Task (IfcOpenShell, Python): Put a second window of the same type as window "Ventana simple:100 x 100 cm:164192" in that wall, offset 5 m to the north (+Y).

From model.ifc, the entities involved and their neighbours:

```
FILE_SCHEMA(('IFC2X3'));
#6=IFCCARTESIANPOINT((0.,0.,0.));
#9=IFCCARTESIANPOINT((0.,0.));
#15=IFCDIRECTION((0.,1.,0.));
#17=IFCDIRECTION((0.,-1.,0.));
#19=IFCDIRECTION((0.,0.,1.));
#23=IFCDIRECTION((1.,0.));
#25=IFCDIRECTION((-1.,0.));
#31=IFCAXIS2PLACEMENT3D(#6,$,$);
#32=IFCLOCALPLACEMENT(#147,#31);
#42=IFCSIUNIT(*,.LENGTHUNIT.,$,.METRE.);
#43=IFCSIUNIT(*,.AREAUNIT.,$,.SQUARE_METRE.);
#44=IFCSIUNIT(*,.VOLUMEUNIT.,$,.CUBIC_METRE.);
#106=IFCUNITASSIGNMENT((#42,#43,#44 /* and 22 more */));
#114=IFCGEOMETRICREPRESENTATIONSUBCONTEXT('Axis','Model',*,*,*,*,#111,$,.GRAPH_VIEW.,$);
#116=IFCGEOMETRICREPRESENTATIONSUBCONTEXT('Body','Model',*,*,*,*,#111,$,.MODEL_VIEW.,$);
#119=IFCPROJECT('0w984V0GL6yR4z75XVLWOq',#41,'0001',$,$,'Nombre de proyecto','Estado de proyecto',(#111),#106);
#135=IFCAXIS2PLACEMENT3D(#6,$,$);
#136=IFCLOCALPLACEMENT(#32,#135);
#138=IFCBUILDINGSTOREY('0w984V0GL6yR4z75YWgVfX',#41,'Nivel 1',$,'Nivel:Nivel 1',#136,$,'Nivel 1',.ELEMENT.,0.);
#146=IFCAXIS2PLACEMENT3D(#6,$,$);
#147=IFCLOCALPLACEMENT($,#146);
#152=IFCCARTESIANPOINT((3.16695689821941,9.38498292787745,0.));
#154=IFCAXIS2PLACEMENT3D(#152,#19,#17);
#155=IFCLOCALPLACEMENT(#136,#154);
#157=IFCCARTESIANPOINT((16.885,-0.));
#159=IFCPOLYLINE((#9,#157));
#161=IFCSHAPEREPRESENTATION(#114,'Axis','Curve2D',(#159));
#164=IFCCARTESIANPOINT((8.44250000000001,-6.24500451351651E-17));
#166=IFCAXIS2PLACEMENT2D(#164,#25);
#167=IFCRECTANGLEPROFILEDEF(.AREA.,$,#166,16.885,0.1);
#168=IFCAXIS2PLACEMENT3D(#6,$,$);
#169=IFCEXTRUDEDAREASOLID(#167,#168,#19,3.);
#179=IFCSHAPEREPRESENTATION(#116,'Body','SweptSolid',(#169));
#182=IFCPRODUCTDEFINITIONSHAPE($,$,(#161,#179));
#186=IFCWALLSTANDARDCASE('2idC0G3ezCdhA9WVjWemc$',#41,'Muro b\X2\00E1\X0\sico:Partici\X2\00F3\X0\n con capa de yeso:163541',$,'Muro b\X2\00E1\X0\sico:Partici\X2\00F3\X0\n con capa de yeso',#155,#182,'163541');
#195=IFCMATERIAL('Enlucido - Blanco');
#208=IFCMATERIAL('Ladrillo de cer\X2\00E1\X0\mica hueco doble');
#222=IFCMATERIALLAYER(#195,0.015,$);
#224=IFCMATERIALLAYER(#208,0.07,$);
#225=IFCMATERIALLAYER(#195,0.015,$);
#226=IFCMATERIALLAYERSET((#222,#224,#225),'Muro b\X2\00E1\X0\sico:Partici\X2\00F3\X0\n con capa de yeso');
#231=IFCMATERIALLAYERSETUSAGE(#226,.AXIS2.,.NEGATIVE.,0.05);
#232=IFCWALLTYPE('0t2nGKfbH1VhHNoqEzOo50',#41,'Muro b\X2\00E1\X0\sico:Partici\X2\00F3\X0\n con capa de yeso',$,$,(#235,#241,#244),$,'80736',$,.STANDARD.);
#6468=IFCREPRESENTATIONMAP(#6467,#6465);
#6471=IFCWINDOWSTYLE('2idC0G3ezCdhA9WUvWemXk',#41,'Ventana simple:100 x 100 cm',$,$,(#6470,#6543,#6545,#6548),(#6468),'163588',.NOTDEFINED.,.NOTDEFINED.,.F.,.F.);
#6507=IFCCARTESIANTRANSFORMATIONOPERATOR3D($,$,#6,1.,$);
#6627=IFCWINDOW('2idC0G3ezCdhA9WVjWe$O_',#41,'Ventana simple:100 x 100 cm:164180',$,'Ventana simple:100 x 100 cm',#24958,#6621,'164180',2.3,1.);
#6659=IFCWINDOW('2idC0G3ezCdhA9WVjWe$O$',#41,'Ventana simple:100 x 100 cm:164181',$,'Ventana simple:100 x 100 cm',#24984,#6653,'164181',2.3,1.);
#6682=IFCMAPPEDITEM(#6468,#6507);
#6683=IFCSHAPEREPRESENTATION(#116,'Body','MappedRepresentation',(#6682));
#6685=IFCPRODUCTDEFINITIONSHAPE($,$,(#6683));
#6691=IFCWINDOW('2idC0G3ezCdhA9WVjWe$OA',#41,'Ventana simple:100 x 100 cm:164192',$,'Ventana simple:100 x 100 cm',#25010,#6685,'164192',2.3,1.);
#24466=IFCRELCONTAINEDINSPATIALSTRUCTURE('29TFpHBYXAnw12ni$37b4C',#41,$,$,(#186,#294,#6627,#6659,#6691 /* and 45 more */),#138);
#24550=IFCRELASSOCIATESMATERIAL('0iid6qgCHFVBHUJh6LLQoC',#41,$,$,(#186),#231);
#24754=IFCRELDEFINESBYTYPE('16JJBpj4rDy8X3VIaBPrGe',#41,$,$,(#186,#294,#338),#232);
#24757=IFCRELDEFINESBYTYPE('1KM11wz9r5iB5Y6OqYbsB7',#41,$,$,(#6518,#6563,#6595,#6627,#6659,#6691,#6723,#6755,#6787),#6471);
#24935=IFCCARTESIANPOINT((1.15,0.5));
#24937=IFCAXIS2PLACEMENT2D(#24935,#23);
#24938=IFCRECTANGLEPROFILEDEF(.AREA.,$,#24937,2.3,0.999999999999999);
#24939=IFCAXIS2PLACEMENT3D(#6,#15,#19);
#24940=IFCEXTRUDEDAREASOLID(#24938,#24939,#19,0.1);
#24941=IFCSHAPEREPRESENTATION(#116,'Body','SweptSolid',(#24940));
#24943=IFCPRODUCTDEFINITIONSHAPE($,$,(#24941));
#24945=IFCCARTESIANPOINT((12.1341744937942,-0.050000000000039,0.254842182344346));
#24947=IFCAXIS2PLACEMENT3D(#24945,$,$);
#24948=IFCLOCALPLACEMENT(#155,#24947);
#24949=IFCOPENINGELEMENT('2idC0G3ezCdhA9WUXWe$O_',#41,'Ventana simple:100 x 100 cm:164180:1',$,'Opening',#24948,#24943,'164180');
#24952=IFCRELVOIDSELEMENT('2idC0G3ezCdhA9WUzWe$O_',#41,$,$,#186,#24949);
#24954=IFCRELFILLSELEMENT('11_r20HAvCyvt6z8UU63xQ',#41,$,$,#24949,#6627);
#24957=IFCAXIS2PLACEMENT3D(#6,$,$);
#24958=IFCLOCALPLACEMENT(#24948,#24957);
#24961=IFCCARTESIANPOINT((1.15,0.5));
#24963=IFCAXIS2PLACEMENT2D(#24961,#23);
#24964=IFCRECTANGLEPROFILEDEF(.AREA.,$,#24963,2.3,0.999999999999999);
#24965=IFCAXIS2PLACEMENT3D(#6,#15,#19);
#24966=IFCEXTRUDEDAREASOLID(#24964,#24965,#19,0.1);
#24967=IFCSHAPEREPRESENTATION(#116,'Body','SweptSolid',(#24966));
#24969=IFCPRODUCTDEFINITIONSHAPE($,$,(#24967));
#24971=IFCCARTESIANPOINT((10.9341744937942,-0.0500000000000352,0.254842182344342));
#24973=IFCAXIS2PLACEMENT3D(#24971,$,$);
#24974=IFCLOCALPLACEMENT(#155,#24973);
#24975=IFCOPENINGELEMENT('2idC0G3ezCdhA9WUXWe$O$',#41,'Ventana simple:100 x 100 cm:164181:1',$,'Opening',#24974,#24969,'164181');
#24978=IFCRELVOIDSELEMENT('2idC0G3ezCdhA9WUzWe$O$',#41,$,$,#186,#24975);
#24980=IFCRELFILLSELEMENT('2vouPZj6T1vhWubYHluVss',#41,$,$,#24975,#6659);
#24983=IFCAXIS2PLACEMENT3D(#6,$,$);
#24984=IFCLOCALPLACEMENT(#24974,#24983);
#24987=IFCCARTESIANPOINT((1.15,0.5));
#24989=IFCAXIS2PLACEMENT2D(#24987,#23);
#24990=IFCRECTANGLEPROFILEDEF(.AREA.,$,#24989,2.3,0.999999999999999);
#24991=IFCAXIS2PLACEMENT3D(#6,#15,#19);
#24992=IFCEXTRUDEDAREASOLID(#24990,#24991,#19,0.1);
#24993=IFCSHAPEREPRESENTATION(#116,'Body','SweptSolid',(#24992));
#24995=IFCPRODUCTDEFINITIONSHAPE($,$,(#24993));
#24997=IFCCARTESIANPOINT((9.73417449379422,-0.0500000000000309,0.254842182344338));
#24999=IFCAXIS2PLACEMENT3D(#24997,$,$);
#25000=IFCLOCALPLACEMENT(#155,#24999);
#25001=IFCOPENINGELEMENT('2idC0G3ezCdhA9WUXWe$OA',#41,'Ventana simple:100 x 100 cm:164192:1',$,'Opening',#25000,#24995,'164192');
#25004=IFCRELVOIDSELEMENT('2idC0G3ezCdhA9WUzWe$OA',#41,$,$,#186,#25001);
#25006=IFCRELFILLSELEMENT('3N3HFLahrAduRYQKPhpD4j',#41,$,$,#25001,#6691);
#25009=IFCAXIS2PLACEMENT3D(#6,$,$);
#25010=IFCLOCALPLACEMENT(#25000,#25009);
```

```python
import ifcopenshell
import ifcopenshell.api.feature
import ifcopenshell.api.geometry
import ifcopenshell.api.root
import ifcopenshell.geom
import ifcopenshell.util.element
import ifcopenshell.util.placement
import ifcopenshell.util.shape

model = ifcopenshell.open("model.ifc")
settings = ifcopenshell.geom.settings()


def volume(element):
    """Net volume in cubic metres, openings subtracted."""
    shape = ifcopenshell.geom.create_shape(settings, element)
    return ifcopenshell.util.shape.get_volume(shape.geometry)


def reuse_history(source, copy):
    """copy_class also copies each property set's owner history, people and application; keep the originals."""
    for rel in copy.IsDefinedBy:
        if rel.is_a("IfcRelDefinesByProperties") and (history := rel.RelatingPropertyDefinition.OwnerHistory):
            rel.RelatingPropertyDefinition.OwnerHistory = source.OwnerHistory
            ifcopenshell.util.element.remove_deep2(model, history)


window = model.by_guid("2idC0G3ezCdhA9WVjWe$OA")
opening = window.FillsVoids[0].RelatingOpeningElement
wall = opening.VoidsElements[0].RelatingBuildingElement
before = volume(wall)
shift = ifcopenshell.util.placement.get_local_placement(wall.ObjectPlacement)[:3, 0] * -5.0

# copy_class copies the void relationship, type, container and properties, but no geometry.
new_opening = ifcopenshell.api.root.copy_class(model, product=opening)
new_opening.Representation = ifcopenshell.util.element.copy_deep(
    model, opening.Representation, exclude=["IfcGeometricRepresentationContext", "IfcRepresentationMap"]
)
new_opening.Name = "Ventana simple:100 x 100 cm"
new_opening.Tag = None
new_window = ifcopenshell.api.root.copy_class(model, product=window)
new_window.Representation = ifcopenshell.util.element.copy_deep(
    model, window.Representation, exclude=["IfcGeometricRepresentationContext", "IfcRepresentationMap"]
)
new_window.Name = "Ventana simple:100 x 100 cm"
new_window.Tag = None
reuse_history(window, new_window)
fills = ifcopenshell.api.feature.add_filling(model, opening=new_opening, element=new_window)
fills.OwnerHistory = new_window.OwnerHistory  # required in IFC2X3

for old, new in ((opening, new_opening), (window, new_window)):
    matrix = ifcopenshell.util.placement.get_local_placement(old.ObjectPlacement)
    matrix[:3, 3] += shift
    ifcopenshell.api.geometry.edit_object_placement(model, product=new, matrix=matrix, is_si=False)

after = volume(wall)

print(f"wall volume {before:.3f} -> {after:.3f} m3")

model.write("model_updated.ifc")
```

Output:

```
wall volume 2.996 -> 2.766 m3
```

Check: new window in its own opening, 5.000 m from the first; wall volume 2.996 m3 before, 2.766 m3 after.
